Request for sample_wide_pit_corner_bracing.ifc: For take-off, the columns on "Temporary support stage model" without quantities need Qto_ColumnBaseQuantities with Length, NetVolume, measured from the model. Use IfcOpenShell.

First a look at what the model holds.

```python
import ifcopenshell
import ifcopenshell.util.element
import ifcopenshell.util.unit

model = ifcopenshell.open("sample_wide_pit_corner_bracing.ifc")
print(model.schema)
for unit_type in ("LENGTHUNIT", "AREAUNIT", "VOLUMEUNIT"):
    print(unit_type, ifcopenshell.util.unit.calculate_unit_scale(model, unit_type))
storey = next(s for s in model.by_type("IfcBuildingStorey") if s.Name == "Temporary support stage model")
columns = [e for e in ifcopenshell.util.element.get_decomposition(storey) if e.is_a("IfcColumn")]
for e in sorted(columns, key=lambda e: e.id()):
    print(e.id(), e.is_a(), e.Name, list(ifcopenshell.util.element.get_psets(e, qtos_only=True)), sep=" | ")
```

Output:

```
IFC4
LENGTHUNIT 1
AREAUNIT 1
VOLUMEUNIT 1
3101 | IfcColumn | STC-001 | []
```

```python
import ifcopenshell
import ifcopenshell.api.pset
import ifcopenshell.geom
import ifcopenshell.util.element
import ifcopenshell.util.shape
import ifcopenshell.util.unit

model = ifcopenshell.open("sample_wide_pit_corner_bracing.ifc")
unit_scale = ifcopenshell.util.unit.calculate_unit_scale(model)
volume_scale = ifcopenshell.util.unit.calculate_unit_scale(model, "VOLUMEUNIT")
settings = ifcopenshell.geom.settings()

storey = next(s for s in model.by_type("IfcBuildingStorey") if s.Name == "Temporary support stage model")
columns = [e for e in ifcopenshell.util.element.get_decomposition(storey) if e.is_a("IfcColumn")]

for e in sorted(columns, key=lambda e: e.id()):
    if ifcopenshell.util.element.get_psets(e, qtos_only=True, should_inherit=False):
        continue
    # Geometry comes back in metres, in the element's own axes.
    shape = ifcopenshell.geom.create_shape(settings, e)
    values = {
        "Length": ifcopenshell.util.shape.get_z(shape.geometry) / unit_scale,
        "NetVolume": ifcopenshell.util.shape.get_volume(shape.geometry) / volume_scale,
    }
    qto = ifcopenshell.api.pset.add_qto(model, product=e, name="Qto_ColumnBaseQuantities")
    ifcopenshell.api.pset.edit_qto(model, qto=qto, properties=values)
    print(e.id(), {k: round(v, 3) for k, v in values.items()})

model.write("sample_wide_pit_corner_bracing_v2.ifc")
```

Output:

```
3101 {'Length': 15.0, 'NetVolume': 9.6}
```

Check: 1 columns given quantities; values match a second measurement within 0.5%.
